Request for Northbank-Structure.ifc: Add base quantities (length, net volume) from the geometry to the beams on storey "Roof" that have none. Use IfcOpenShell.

First a look at what the model holds.

```python
import ifcopenshell
import ifcopenshell.util.element
import ifcopenshell.util.unit

model = ifcopenshell.open("Northbank-Structure.ifc")
print(model.schema)
for unit_type in ("LENGTHUNIT", "AREAUNIT", "VOLUMEUNIT"):
    print(unit_type, ifcopenshell.util.unit.calculate_unit_scale(model, unit_type))
storey = next(s for s in model.by_type("IfcBuildingStorey") if s.Name == "Roof")
beams = [e for e in ifcopenshell.util.element.get_decomposition(storey) if e.is_a("IfcBeam")]
for e in sorted(beams, key=lambda e: e.id()):
    print(e.id(), e.is_a(), e.Name, list(ifcopenshell.util.element.get_psets(e, qtos_only=True)), sep=" | ")
```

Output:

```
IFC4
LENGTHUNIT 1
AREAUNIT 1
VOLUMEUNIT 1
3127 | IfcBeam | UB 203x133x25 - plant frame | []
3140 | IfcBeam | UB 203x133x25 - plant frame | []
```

```python
import ifcopenshell
import ifcopenshell.api.pset
import ifcopenshell.geom
import ifcopenshell.util.element
import ifcopenshell.util.shape
import ifcopenshell.util.unit

model = ifcopenshell.open("Northbank-Structure.ifc")
unit_scale = ifcopenshell.util.unit.calculate_unit_scale(model)
volume_scale = ifcopenshell.util.unit.calculate_unit_scale(model, "VOLUMEUNIT")
settings = ifcopenshell.geom.settings()

storey = next(s for s in model.by_type("IfcBuildingStorey") if s.Name == "Roof")
beams = [e for e in ifcopenshell.util.element.get_decomposition(storey) if e.is_a("IfcBeam")]

for e in sorted(beams, key=lambda e: e.id()):
    if ifcopenshell.util.element.get_psets(e, qtos_only=True, should_inherit=False):
        continue
    # Geometry comes back in metres, in the element's own axes.
    shape = ifcopenshell.geom.create_shape(settings, e)
    values = {
        "Length": ifcopenshell.util.shape.get_max_xyz(shape.geometry) / unit_scale,
        "NetVolume": ifcopenshell.util.shape.get_volume(shape.geometry) / volume_scale,
    }
    qto = ifcopenshell.api.pset.add_qto(model, product=e, name="Qto_BeamBaseQuantities")
    ifcopenshell.api.pset.edit_qto(model, qto=qto, properties=values)
    print(e.id(), {k: round(v, 3) for k, v in values.items()})

model.write("Northbank-Structure-out.ifc")
```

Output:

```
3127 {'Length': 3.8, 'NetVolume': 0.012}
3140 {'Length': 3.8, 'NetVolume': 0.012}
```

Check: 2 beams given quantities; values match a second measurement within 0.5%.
